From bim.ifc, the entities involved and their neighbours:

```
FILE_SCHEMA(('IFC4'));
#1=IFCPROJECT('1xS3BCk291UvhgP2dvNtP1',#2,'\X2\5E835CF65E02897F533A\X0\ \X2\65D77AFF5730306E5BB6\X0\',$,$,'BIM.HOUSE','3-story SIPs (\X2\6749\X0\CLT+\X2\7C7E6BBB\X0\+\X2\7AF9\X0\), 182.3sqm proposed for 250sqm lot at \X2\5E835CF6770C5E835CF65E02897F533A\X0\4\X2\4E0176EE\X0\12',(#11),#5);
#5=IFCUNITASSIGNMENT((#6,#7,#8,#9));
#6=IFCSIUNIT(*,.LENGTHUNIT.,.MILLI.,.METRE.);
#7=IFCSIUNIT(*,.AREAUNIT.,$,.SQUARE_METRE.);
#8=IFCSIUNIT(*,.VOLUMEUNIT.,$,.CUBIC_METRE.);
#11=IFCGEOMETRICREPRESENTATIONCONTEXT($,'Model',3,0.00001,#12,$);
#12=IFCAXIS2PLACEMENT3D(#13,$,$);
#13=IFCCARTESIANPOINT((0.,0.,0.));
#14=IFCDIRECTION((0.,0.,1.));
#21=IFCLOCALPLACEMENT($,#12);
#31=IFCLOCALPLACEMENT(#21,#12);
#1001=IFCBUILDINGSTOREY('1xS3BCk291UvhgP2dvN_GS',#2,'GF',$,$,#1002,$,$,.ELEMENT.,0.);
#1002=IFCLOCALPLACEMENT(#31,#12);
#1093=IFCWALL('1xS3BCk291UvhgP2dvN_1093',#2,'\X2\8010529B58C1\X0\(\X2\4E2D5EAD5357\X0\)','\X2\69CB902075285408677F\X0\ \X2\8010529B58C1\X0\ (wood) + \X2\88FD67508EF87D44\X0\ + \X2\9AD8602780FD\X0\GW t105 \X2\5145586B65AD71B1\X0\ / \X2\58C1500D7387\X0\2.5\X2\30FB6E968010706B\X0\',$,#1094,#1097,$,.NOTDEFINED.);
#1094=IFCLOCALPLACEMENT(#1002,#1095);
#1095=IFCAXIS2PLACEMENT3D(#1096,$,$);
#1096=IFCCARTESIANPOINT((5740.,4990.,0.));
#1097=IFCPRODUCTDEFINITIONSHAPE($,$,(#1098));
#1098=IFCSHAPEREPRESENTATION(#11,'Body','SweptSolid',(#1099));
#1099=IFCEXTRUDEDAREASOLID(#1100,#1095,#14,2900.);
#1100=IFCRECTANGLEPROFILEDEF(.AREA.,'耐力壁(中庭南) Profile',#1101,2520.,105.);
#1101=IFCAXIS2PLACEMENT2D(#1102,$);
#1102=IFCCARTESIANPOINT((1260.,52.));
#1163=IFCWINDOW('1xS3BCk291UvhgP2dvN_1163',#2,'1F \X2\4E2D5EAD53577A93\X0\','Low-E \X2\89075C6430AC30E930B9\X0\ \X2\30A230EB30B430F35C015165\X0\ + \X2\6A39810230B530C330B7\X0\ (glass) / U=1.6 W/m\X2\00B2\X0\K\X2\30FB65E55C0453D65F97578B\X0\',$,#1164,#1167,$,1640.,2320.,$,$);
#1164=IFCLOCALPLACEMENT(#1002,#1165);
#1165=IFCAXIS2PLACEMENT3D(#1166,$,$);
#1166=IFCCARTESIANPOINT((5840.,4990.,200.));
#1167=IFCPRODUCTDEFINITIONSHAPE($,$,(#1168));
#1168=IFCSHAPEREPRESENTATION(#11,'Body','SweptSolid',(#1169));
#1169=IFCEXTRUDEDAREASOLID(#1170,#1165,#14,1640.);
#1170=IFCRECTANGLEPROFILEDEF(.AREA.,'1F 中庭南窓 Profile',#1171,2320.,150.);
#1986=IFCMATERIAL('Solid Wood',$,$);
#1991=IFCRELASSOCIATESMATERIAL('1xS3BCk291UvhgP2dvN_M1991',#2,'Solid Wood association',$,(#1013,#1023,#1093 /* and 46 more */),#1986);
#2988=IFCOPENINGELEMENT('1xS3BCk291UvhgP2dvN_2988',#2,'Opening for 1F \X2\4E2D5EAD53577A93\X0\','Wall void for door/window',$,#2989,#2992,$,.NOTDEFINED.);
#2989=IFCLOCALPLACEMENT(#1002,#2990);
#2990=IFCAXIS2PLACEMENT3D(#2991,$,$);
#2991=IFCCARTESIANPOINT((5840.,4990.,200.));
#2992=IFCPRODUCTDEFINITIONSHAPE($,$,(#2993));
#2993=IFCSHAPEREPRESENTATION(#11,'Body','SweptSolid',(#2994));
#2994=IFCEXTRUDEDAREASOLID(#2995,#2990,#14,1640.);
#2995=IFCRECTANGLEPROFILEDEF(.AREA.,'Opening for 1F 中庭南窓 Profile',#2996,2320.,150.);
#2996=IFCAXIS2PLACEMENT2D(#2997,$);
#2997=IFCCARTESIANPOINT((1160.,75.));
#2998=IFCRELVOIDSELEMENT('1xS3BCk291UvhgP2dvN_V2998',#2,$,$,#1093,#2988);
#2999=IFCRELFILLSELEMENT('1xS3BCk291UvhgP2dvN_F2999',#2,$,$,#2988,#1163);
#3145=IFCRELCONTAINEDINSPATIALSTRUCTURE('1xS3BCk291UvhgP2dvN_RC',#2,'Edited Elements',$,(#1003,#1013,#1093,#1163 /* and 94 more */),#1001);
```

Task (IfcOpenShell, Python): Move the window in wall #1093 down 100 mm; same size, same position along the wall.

```python
import numpy as np
import ifcopenshell
import ifcopenshell.api.geometry
import ifcopenshell.util.placement
import ifcopenshell.util.unit

model = ifcopenshell.open("bim.ifc")
unit_scale = ifcopenshell.util.unit.calculate_unit_scale(model)

window = model.by_id(1163)
opening = window.FillsVoids[0].RelatingOpeningElement
dz = -0.1 / unit_scale

shift = np.array([0.0, 0.0, dz])
# The window is not placed relative to its opening, so move both.
for product in (opening, window):
    matrix = ifcopenshell.util.placement.get_local_placement(product.ObjectPlacement)
    matrix[:3, 3] += shift
    ifcopenshell.api.geometry.edit_object_placement(model, product=product, matrix=matrix, is_si=False)

print(f"moved by {dz * unit_scale:+.3f} m")

model.write("bim_updated.ifc")
```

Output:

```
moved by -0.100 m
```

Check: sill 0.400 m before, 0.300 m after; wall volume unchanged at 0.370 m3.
